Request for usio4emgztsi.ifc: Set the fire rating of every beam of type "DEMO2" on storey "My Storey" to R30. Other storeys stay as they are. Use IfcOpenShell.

First a look at what the model holds.

```python
import ifcopenshell
import ifcopenshell.util.element

model = ifcopenshell.open("usio4emgztsi.ifc")
print(model.schema)
storey = next(s for s in model.by_type("IfcBuildingStorey") if s.Name == "My Storey")
beams = [e for e in ifcopenshell.util.element.get_decomposition(storey) if e.is_a("IfcBeam")]
seen = {}
for e in beams:
    element_type = ifcopenshell.util.element.get_type(e)
    key = (element_type.Name if element_type != e and element_type else None, ifcopenshell.util.element.get_pset(e, "Pset_BeamCommon", "FireRating"))
    seen[key] = seen.get(key, 0) + 1
for (name, value), count in sorted(seen.items(), key=str):
    print(count, "x", name, "|", value)
```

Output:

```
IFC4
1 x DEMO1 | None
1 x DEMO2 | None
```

```python
import ifcopenshell
import ifcopenshell.api.pset
import ifcopenshell.util.element

model = ifcopenshell.open("usio4emgztsi.ifc")

storey = next(s for s in model.by_type("IfcBuildingStorey") if s.Name == "My Storey")
beams = [e for e in ifcopenshell.util.element.get_decomposition(storey) if e.is_a("IfcBeam")]

count = 0
for e in beams:
    element_type = ifcopenshell.util.element.get_type(e)
    if element_type in (None, e) or element_type.Name != "DEMO2":
        continue
    # add_pset returns the element's existing set when there is one.
    pset = ifcopenshell.api.pset.add_pset(model, product=e, name="Pset_BeamCommon")
    ifcopenshell.api.pset.edit_pset(model, pset=pset, properties={"FireRating": "R30"})
    count += 1

print(count, "beams updated")

model.write("usio4emgztsi-out.ifc")
```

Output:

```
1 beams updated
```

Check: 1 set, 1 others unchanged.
